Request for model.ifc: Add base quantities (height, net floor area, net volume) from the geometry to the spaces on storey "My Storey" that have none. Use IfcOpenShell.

First a look at what the model holds.

```python
import ifcopenshell
import ifcopenshell.util.element
import ifcopenshell.util.unit

model = ifcopenshell.open("model.ifc")
print(model.schema)
for unit_type in ("LENGTHUNIT", "AREAUNIT", "VOLUMEUNIT"):
    print(unit_type, ifcopenshell.util.unit.calculate_unit_scale(model, unit_type))
storey = next(s for s in model.by_type("IfcBuildingStorey") if s.Name == "My Storey")
spaces = [e for e in ifcopenshell.util.element.get_decomposition(storey) if e.is_a("IfcSpace")]
for e in sorted(spaces, key=lambda e: e.id()):
    print(e.id(), e.is_a(), e.Name, list(ifcopenshell.util.element.get_psets(e, qtos_only=True)), sep=" | ")
```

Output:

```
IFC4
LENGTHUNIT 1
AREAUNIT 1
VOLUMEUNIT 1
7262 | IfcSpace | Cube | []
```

```python
import ifcopenshell
import ifcopenshell.api.pset
import ifcopenshell.geom
import ifcopenshell.util.element
import ifcopenshell.util.shape
import ifcopenshell.util.unit

model = ifcopenshell.open("model.ifc")
unit_scale = ifcopenshell.util.unit.calculate_unit_scale(model)
area_scale = ifcopenshell.util.unit.calculate_unit_scale(model, "AREAUNIT")
volume_scale = ifcopenshell.util.unit.calculate_unit_scale(model, "VOLUMEUNIT")
settings = ifcopenshell.geom.settings()

storey = next(s for s in model.by_type("IfcBuildingStorey") if s.Name == "My Storey")
spaces = [e for e in ifcopenshell.util.element.get_decomposition(storey) if e.is_a("IfcSpace")]

for e in sorted(spaces, key=lambda e: e.id()):
    if ifcopenshell.util.element.get_psets(e, qtos_only=True, should_inherit=False):
        continue
    # Geometry comes back in metres, in the element's own axes.
    shape = ifcopenshell.geom.create_shape(settings, e)
    values = {
        "Height": ifcopenshell.util.shape.get_z(shape.geometry) / unit_scale,
        "NetFloorArea": ifcopenshell.util.shape.get_footprint_area(shape.geometry) / area_scale,
        "NetVolume": ifcopenshell.util.shape.get_volume(shape.geometry) / volume_scale,
    }
    qto = ifcopenshell.api.pset.add_qto(model, product=e, name="Qto_SpaceBaseQuantities")
    ifcopenshell.api.pset.edit_qto(model, qto=qto, properties=values)
    print(e.id(), {k: round(v, 3) for k, v in values.items()})

model.write("model-out.ifc")
```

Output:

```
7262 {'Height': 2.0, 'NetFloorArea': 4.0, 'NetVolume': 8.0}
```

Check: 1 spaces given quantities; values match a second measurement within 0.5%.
